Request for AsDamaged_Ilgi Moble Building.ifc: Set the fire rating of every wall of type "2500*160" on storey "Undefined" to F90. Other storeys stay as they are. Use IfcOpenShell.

First a look at what the model holds.

```python
import ifcopenshell
import ifcopenshell.util.element

model = ifcopenshell.open("AsDamaged_Ilgi Moble Building.ifc")
print(model.schema)
storey = next(s for s in model.by_type("IfcBuildingStorey") if s.Name == "Undefined")
walls = [e for e in ifcopenshell.util.element.get_decomposition(storey) if e.is_a("IfcWall")]
seen = {}
for e in walls:
    element_type = ifcopenshell.util.element.get_type(e)
    key = (element_type.Name if element_type != e and element_type else None, ifcopenshell.util.element.get_pset(e, "Pset_WallCommon", "FireRating"))
    seen[key] = seen.get(key, 0) + 1
for (name, value), count in sorted(seen.items(), key=str):
    print(count, "x", name, "|", value)
```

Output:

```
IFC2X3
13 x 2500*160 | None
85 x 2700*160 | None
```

```python
import ifcopenshell
import ifcopenshell.api.pset
import ifcopenshell.util.element

model = ifcopenshell.open("AsDamaged_Ilgi Moble Building.ifc")

storey = next(s for s in model.by_type("IfcBuildingStorey") if s.Name == "Undefined")
walls = [e for e in ifcopenshell.util.element.get_decomposition(storey) if e.is_a("IfcWall")]

count = 0
for e in walls:
    element_type = ifcopenshell.util.element.get_type(e)
    if element_type in (None, e) or element_type.Name != "2500*160":
        continue
    # add_pset returns the element's existing set when there is one.
    pset = ifcopenshell.api.pset.add_pset(model, product=e, name="Pset_WallCommon")
    ifcopenshell.api.pset.edit_pset(model, pset=pset, properties={"FireRating": "F90"})
    count += 1

print(count, "walls updated")

model.write("AsDamaged_Ilgi Moble Building_edited.ifc")
```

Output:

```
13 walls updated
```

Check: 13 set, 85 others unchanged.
